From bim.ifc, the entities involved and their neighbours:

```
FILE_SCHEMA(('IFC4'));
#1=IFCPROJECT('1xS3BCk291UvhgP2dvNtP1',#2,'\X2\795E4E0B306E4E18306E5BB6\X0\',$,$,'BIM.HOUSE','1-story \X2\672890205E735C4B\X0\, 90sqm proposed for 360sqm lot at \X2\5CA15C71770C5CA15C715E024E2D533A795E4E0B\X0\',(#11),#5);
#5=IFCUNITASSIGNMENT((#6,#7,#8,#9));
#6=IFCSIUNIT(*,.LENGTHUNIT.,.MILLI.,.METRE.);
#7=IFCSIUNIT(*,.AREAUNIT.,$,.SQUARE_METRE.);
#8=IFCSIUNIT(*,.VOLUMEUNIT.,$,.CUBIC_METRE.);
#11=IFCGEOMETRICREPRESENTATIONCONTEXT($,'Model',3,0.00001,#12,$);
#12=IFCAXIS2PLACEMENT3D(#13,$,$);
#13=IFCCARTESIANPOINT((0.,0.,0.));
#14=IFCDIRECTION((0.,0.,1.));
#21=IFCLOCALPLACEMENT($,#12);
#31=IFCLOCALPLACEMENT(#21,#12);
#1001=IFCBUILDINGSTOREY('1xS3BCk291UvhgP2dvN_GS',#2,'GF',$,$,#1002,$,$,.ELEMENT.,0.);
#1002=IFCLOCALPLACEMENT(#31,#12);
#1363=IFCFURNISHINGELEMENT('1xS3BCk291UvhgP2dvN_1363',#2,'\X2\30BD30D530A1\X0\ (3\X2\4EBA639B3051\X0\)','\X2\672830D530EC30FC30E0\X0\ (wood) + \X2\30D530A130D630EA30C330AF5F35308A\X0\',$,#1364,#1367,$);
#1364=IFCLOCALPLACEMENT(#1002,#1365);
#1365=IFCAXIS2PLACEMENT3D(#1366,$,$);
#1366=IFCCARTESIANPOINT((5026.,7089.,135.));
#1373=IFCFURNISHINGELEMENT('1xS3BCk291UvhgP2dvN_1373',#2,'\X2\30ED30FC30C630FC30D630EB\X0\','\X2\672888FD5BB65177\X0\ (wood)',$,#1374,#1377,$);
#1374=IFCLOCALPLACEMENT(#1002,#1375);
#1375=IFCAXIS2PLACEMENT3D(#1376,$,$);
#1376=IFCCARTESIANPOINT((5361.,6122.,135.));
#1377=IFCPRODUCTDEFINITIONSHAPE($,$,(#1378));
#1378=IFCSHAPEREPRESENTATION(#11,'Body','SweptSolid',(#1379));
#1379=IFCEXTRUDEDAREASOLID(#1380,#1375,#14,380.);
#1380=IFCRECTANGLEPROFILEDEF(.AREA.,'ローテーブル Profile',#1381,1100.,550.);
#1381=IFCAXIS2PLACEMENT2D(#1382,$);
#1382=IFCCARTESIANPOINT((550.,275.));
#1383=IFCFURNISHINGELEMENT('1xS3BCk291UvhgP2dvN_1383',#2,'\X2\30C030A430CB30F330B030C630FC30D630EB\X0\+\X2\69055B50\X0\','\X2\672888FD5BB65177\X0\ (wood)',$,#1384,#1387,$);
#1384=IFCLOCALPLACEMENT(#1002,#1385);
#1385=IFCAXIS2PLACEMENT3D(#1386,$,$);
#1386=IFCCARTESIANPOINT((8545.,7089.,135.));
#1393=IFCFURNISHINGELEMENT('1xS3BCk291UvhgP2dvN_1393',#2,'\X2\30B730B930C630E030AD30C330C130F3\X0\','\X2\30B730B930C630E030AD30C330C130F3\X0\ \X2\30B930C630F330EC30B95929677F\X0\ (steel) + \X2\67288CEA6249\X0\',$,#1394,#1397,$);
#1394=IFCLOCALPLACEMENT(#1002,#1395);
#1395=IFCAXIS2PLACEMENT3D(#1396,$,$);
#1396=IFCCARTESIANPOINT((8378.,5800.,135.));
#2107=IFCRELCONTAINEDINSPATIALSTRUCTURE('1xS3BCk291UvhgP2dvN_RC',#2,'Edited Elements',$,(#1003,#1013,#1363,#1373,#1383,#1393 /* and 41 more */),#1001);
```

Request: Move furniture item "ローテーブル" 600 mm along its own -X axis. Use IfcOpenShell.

```python
import ifcopenshell
import ifcopenshell.api.geometry
import ifcopenshell.util.placement
import ifcopenshell.util.unit

model = ifcopenshell.open("bim.ifc")
unit_scale = ifcopenshell.util.unit.calculate_unit_scale(model)

item = model.by_guid("1xS3BCk291UvhgP2dvN_1373")
matrix = ifcopenshell.util.placement.get_local_placement(item.ObjectPlacement)
matrix[:3, 3] -= matrix[:3, 0] * 0.6 / unit_scale
ifcopenshell.api.geometry.edit_object_placement(model, product=item, matrix=matrix, is_si=False)

print(ifcopenshell.util.placement.get_local_placement(item.ObjectPlacement).round(3) + 0.0)

model.write("bim-out.ifc")
```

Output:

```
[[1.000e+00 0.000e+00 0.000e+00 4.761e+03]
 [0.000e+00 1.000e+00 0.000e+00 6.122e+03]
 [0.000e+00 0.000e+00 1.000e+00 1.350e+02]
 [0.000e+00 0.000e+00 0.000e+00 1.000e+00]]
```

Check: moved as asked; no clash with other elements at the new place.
